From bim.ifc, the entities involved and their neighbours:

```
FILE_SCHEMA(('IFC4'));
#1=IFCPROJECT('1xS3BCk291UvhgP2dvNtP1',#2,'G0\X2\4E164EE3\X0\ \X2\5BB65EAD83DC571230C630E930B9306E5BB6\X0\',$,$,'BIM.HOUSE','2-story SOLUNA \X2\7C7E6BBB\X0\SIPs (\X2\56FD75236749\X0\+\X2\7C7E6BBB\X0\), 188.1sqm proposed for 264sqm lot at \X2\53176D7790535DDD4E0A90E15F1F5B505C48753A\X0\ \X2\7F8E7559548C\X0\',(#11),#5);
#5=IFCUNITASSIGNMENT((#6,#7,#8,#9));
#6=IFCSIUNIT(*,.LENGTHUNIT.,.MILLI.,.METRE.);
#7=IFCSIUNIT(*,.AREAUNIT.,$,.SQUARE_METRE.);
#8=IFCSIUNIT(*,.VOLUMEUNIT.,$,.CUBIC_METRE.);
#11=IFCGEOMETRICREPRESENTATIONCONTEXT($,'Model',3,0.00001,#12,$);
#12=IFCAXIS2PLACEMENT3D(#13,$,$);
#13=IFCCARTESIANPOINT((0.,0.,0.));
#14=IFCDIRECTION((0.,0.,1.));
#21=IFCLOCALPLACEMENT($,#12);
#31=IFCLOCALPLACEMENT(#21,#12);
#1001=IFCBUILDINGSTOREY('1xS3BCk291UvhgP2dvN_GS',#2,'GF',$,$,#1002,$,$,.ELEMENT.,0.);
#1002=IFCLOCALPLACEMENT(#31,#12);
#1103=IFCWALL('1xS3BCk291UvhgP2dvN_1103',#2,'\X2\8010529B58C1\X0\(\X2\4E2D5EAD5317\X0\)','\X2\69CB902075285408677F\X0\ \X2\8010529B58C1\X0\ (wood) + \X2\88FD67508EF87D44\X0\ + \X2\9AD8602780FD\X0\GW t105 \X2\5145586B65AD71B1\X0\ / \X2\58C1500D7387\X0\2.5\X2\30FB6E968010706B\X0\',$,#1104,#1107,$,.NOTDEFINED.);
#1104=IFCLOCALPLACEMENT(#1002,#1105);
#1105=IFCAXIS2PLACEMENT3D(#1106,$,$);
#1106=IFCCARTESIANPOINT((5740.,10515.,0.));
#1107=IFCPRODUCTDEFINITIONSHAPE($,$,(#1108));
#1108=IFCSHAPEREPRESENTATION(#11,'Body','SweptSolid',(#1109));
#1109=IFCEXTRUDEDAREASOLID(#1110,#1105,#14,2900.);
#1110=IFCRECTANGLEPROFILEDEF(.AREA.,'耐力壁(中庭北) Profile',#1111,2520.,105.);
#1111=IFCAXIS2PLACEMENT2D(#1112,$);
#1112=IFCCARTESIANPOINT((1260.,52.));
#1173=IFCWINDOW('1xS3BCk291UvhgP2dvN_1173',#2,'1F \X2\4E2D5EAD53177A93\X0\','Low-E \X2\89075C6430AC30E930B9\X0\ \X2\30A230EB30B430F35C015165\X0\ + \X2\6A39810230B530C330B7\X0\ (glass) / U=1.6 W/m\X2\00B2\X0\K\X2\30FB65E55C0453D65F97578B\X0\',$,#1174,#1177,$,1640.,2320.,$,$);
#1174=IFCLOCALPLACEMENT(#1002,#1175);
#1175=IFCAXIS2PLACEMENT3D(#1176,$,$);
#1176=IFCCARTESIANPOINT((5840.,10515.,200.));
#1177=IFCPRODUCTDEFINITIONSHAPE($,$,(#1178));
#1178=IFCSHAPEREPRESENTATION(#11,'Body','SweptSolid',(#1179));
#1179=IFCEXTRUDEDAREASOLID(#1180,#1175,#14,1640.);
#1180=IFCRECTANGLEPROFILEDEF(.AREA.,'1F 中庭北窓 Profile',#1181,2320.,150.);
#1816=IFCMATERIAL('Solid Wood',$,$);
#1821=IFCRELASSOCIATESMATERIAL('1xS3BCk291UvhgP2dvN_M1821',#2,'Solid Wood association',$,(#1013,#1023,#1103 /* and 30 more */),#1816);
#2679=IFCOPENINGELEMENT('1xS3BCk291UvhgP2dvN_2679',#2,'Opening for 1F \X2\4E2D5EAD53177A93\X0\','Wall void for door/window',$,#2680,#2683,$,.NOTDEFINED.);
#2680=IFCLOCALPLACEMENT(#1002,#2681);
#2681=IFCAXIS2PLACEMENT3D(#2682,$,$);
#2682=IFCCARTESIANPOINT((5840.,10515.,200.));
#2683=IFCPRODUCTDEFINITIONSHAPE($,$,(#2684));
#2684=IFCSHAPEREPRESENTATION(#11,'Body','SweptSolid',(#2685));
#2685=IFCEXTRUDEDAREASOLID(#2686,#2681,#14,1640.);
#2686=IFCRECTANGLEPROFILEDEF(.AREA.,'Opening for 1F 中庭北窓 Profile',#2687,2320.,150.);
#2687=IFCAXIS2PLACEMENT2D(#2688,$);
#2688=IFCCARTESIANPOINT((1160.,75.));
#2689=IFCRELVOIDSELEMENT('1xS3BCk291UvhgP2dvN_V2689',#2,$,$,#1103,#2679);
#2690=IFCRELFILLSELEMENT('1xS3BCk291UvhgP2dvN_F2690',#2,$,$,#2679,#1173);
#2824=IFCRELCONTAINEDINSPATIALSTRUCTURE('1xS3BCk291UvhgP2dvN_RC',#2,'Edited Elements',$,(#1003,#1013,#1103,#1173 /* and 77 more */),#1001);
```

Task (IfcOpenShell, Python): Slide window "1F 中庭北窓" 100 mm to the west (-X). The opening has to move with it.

```python
import ifcopenshell
import ifcopenshell.api.geometry
import ifcopenshell.util.placement
import ifcopenshell.util.unit

model = ifcopenshell.open("bim.ifc")
unit_scale = ifcopenshell.util.unit.calculate_unit_scale(model)

window = model.by_id(1173)
opening = window.FillsVoids[0].RelatingOpeningElement
wall = opening.VoidsElements[0].RelatingBuildingElement

wall_matrix = ifcopenshell.util.placement.get_local_placement(wall.ObjectPlacement)
shift = wall_matrix[:3, 0] * -0.1 / unit_scale
before = ifcopenshell.util.placement.get_local_placement(window.ObjectPlacement)[:3, 3].copy()

# The window is not placed relative to its opening, so move both.
for product in (opening, window):
    matrix = ifcopenshell.util.placement.get_local_placement(product.ObjectPlacement)
    matrix[:3, 3] += shift
    ifcopenshell.api.geometry.edit_object_placement(model, product=product, matrix=matrix, is_si=False)

after = ifcopenshell.util.placement.get_local_placement(window.ObjectPlacement)[:3, 3]
print("window moved by", (after - before).round(3) + 0.0)

model.write("bim_edited.ifc")
```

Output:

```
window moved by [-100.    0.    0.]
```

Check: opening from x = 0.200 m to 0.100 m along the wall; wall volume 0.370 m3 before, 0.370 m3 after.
